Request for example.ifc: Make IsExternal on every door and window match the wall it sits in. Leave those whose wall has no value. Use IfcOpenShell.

First a look at what the model holds.

```python
import ifcopenshell
import ifcopenshell.util.element

model = ifcopenshell.open("example.ifc")
print(model.schema)
seen = {}
for e in model.by_type("IfcDoor") + model.by_type("IfcWindow"):
    if not e.FillsVoids:
        continue
    host = e.FillsVoids[0].RelatingOpeningElement.VoidsElements[0].RelatingBuildingElement
    own = ifcopenshell.util.element.get_pset(e, f"Pset_{e.is_a()[3:].removesuffix('StandardCase')}Common", "IsExternal")
    wall = ifcopenshell.util.element.get_pset(host, "Pset_WallCommon", "IsExternal")
    seen[e.is_a(), own, wall] = seen.get((e.is_a(), own, wall), 0) + 1
for (cls, own, wall), count in sorted(seen.items(), key=str):
    print(count, cls, "IsExternal:", own, "| host wall:", wall)
```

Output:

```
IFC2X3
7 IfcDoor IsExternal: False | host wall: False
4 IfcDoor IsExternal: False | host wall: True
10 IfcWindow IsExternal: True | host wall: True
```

```python
import ifcopenshell
import ifcopenshell.api.pset
import ifcopenshell.util.element

model = ifcopenshell.open("example.ifc")

count = 0
for ifc_class, pset_name in (("IfcDoor", "Pset_DoorCommon"), ("IfcWindow", "Pset_WindowCommon")):
    for e in model.by_type(ifc_class):
        if not e.FillsVoids:
            continue
        host = e.FillsVoids[0].RelatingOpeningElement.VoidsElements[0].RelatingBuildingElement
        external = ifcopenshell.util.element.get_pset(host, "Pset_WallCommon", "IsExternal")
        if external is None or ifcopenshell.util.element.get_pset(e, pset_name, "IsExternal") == external:
            continue
        pset = ifcopenshell.api.pset.add_pset(model, product=e, name=pset_name)
        ifcopenshell.api.pset.edit_pset(model, pset=pset, properties={"IsExternal": external})
        count += 1

print(count, "updated")

model.write("example-out.ifc")
```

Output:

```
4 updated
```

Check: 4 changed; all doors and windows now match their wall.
